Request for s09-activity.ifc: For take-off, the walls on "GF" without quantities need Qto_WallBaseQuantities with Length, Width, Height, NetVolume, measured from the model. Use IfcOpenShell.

First a look at what the model holds.

```python
import ifcopenshell
import ifcopenshell.util.element
import ifcopenshell.util.unit

model = ifcopenshell.open("s09-activity.ifc")
print(model.schema)
for unit_type in ("LENGTHUNIT", "AREAUNIT", "VOLUMEUNIT"):
    print(unit_type, ifcopenshell.util.unit.calculate_unit_scale(model, unit_type))
storey = next(s for s in model.by_type("IfcBuildingStorey") if s.Name == "GF")
walls = [e for e in ifcopenshell.util.element.get_decomposition(storey) if e.is_a("IfcWall")]
for e in sorted(walls, key=lambda e: e.id()):
    print(e.id(), e.is_a(), e.Name, list(ifcopenshell.util.element.get_psets(e, qtos_only=True)), sep=" | ")
```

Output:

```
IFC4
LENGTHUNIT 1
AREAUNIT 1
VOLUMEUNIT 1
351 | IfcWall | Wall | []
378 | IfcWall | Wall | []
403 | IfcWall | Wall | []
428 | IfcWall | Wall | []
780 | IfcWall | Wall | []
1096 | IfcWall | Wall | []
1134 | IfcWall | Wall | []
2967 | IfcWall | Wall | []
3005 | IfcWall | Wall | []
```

```python
import ifcopenshell
import ifcopenshell.api.pset
import ifcopenshell.geom
import ifcopenshell.util.element
import ifcopenshell.util.shape
import ifcopenshell.util.unit

model = ifcopenshell.open("s09-activity.ifc")
unit_scale = ifcopenshell.util.unit.calculate_unit_scale(model)
volume_scale = ifcopenshell.util.unit.calculate_unit_scale(model, "VOLUMEUNIT")
settings = ifcopenshell.geom.settings()

storey = next(s for s in model.by_type("IfcBuildingStorey") if s.Name == "GF")
walls = [e for e in ifcopenshell.util.element.get_decomposition(storey) if e.is_a("IfcWall")]

for e in sorted(walls, key=lambda e: e.id()):
    if ifcopenshell.util.element.get_psets(e, qtos_only=True, should_inherit=False):
        continue
    # Geometry comes back in metres, in the element's own axes.
    shape = ifcopenshell.geom.create_shape(settings, e)
    values = {
        "Length": ifcopenshell.util.shape.get_x(shape.geometry) / unit_scale,
        "Width": ifcopenshell.util.shape.get_y(shape.geometry) / unit_scale,
        "Height": ifcopenshell.util.shape.get_z(shape.geometry) / unit_scale,
        "NetVolume": ifcopenshell.util.shape.get_volume(shape.geometry) / volume_scale,
    }
    qto = ifcopenshell.api.pset.add_qto(model, product=e, name="Qto_WallBaseQuantities")
    ifcopenshell.api.pset.edit_qto(model, qto=qto, properties=values)
    print(e.id(), {k: round(v, 3) for k, v in values.items()})

model.write("s09-activity_edited.ifc")
```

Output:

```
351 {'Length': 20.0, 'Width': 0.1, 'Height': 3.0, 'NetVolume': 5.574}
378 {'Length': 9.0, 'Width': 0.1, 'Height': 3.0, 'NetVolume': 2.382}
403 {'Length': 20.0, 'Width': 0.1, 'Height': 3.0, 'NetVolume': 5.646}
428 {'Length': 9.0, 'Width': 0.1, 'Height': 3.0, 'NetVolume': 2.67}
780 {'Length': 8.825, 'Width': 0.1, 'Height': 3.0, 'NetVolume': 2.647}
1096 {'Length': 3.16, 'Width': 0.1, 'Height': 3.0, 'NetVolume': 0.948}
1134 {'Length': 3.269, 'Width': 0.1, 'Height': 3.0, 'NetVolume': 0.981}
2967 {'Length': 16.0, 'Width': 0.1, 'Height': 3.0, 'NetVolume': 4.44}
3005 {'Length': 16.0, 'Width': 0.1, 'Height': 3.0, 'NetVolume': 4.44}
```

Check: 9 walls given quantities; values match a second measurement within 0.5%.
